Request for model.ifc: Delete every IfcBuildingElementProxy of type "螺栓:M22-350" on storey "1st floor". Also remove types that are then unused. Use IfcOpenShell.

First a look at what the model holds.

```python
import ifcopenshell
import ifcopenshell.util.element

model = ifcopenshell.open("model.ifc")
print(model.schema)
storey = next(s for s in model.by_type("IfcBuildingStorey") if s.Name == "1st floor")
proxies = [e for e in ifcopenshell.util.element.get_decomposition(storey) if e.is_a("IfcBuildingElementProxy")]
seen = {}
for e in proxies:
    element_type = ifcopenshell.util.element.get_type(e)
    name = element_type.Name if element_type not in (None, e) else None
    seen[name] = seen.get(name, 0) + 1
for name, count in sorted(seen.items(), key=str):
    print(count, "x", name)
```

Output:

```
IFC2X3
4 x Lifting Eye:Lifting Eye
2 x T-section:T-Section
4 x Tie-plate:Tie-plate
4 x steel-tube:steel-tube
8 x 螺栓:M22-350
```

```python
import ifcopenshell
import ifcopenshell.api.root
import ifcopenshell.util.element

model = ifcopenshell.open("model.ifc")

storey = next(s for s in model.by_type("IfcBuildingStorey") if s.Name == "1st floor")
proxies = [e for e in ifcopenshell.util.element.get_decomposition(storey) if e.is_a("IfcBuildingElementProxy")]
targets = [e for e in proxies if (t := ifcopenshell.util.element.get_type(e)) not in (None, e) and t.Name == "螺栓:M22-350"]
types = {ifcopenshell.util.element.get_type(e) for e in targets} - {None, *targets}

for e in targets:
    ifcopenshell.api.root.remove_product(model, product=e)
print(len(targets), "removed")

unused = [t for t in types if not ifcopenshell.util.element.get_types(t)]
for t in unused:
    ifcopenshell.api.root.remove_product(model, product=t)
print(len(unused), "unused types removed")

model.write("model_rev.ifc")
```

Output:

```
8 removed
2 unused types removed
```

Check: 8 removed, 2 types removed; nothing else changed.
